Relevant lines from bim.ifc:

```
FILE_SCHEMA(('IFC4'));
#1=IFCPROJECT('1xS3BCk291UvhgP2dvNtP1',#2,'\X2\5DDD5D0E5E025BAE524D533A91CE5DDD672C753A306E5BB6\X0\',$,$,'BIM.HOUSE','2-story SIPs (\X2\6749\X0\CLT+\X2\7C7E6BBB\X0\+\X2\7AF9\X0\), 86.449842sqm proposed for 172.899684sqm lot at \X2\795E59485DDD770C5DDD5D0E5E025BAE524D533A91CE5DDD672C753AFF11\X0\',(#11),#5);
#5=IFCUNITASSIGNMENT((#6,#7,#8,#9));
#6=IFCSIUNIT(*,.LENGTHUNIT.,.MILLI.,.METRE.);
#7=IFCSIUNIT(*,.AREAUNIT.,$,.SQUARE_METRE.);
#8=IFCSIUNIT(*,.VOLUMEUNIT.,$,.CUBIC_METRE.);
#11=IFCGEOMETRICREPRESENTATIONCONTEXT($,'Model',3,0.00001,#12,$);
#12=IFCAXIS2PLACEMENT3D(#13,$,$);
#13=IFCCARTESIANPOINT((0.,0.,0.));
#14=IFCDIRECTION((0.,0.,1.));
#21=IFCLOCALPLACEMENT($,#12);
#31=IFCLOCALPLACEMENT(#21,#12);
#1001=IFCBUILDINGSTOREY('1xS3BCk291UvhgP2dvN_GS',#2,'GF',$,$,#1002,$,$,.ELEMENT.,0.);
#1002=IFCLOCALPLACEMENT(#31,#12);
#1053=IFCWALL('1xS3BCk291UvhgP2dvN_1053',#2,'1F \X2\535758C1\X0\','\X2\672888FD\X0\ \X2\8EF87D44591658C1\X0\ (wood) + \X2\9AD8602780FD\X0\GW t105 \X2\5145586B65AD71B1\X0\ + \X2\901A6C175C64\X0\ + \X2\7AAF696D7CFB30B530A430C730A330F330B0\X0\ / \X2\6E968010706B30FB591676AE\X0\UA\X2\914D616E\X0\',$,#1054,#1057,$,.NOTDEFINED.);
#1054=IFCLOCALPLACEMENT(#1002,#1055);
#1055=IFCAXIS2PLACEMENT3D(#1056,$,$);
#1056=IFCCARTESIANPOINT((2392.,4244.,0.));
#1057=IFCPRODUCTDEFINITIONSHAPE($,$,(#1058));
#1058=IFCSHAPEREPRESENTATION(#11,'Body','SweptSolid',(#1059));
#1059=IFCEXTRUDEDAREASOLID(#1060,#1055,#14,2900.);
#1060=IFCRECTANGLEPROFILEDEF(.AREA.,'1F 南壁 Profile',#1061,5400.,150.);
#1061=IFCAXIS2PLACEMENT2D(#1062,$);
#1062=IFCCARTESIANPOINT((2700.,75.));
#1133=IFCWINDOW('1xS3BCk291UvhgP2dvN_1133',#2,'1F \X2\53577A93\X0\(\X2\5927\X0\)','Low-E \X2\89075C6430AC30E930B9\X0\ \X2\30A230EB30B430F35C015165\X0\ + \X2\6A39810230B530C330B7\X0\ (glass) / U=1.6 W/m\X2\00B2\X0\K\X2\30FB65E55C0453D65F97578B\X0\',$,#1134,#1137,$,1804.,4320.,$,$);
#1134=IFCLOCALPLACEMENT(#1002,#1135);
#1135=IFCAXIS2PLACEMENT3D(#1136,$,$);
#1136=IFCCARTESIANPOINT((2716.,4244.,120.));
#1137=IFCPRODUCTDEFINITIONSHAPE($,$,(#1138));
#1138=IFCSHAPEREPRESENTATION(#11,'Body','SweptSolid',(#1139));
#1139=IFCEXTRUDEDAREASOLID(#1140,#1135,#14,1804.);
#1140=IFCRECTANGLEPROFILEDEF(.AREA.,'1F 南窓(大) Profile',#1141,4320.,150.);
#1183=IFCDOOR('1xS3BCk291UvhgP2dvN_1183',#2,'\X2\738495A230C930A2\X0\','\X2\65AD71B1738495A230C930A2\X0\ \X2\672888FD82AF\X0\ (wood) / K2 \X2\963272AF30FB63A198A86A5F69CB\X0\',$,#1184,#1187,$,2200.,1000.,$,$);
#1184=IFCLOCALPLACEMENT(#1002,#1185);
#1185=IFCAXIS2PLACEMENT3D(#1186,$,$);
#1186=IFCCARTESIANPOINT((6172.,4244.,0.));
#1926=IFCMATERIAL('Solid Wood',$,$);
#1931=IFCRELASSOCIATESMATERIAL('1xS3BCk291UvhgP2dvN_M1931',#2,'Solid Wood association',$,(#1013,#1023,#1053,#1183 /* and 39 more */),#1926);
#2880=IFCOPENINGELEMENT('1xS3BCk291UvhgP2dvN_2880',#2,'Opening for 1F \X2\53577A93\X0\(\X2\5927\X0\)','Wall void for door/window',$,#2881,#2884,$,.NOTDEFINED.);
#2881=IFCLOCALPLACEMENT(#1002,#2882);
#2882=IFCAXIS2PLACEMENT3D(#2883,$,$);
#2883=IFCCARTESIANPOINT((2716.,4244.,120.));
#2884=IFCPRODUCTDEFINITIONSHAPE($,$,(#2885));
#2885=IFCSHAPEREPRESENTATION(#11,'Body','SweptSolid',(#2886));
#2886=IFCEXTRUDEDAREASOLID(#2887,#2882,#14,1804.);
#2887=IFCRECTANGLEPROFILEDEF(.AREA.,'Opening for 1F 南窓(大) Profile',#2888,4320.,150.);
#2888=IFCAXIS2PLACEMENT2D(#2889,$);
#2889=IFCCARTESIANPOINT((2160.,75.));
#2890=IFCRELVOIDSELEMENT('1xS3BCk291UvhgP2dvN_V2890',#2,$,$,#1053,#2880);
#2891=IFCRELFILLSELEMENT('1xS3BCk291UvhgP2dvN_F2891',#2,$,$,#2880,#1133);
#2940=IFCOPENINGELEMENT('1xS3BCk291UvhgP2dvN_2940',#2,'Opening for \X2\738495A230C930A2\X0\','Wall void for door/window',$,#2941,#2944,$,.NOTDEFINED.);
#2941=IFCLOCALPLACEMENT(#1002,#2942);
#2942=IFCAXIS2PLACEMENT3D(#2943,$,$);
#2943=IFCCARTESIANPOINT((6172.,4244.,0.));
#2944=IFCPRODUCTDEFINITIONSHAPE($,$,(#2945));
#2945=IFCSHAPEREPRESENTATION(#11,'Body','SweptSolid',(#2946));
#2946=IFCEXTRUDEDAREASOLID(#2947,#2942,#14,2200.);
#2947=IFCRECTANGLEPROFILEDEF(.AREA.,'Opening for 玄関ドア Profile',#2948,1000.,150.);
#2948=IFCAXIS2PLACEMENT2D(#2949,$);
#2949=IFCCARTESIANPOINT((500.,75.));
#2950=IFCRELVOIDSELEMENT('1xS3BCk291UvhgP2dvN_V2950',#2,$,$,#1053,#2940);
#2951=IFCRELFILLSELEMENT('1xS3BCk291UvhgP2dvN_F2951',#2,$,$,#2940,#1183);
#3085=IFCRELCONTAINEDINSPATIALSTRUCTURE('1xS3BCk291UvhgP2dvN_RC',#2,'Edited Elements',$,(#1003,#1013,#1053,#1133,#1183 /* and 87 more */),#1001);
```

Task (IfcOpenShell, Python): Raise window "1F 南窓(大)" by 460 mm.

```python
import numpy as np
import ifcopenshell
import ifcopenshell.api.geometry
import ifcopenshell.util.placement
import ifcopenshell.util.unit

model = ifcopenshell.open("bim.ifc")
unit_scale = ifcopenshell.util.unit.calculate_unit_scale(model)

window = model.by_guid("1xS3BCk291UvhgP2dvN_1133")
opening = window.FillsVoids[0].RelatingOpeningElement
dz = 460.0

shift = np.array([0.0, 0.0, dz])
# The window is not placed relative to its opening, so move both.
for product in (opening, window):
    matrix = ifcopenshell.util.placement.get_local_placement(product.ObjectPlacement)
    matrix[:3, 3] += shift
    ifcopenshell.api.geometry.edit_object_placement(model, product=product, matrix=matrix, is_si=False)

print(f"moved by {dz * unit_scale:+.3f} m")

model.write("bim_v2.ifc")
```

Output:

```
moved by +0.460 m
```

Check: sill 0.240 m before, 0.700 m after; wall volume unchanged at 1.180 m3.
